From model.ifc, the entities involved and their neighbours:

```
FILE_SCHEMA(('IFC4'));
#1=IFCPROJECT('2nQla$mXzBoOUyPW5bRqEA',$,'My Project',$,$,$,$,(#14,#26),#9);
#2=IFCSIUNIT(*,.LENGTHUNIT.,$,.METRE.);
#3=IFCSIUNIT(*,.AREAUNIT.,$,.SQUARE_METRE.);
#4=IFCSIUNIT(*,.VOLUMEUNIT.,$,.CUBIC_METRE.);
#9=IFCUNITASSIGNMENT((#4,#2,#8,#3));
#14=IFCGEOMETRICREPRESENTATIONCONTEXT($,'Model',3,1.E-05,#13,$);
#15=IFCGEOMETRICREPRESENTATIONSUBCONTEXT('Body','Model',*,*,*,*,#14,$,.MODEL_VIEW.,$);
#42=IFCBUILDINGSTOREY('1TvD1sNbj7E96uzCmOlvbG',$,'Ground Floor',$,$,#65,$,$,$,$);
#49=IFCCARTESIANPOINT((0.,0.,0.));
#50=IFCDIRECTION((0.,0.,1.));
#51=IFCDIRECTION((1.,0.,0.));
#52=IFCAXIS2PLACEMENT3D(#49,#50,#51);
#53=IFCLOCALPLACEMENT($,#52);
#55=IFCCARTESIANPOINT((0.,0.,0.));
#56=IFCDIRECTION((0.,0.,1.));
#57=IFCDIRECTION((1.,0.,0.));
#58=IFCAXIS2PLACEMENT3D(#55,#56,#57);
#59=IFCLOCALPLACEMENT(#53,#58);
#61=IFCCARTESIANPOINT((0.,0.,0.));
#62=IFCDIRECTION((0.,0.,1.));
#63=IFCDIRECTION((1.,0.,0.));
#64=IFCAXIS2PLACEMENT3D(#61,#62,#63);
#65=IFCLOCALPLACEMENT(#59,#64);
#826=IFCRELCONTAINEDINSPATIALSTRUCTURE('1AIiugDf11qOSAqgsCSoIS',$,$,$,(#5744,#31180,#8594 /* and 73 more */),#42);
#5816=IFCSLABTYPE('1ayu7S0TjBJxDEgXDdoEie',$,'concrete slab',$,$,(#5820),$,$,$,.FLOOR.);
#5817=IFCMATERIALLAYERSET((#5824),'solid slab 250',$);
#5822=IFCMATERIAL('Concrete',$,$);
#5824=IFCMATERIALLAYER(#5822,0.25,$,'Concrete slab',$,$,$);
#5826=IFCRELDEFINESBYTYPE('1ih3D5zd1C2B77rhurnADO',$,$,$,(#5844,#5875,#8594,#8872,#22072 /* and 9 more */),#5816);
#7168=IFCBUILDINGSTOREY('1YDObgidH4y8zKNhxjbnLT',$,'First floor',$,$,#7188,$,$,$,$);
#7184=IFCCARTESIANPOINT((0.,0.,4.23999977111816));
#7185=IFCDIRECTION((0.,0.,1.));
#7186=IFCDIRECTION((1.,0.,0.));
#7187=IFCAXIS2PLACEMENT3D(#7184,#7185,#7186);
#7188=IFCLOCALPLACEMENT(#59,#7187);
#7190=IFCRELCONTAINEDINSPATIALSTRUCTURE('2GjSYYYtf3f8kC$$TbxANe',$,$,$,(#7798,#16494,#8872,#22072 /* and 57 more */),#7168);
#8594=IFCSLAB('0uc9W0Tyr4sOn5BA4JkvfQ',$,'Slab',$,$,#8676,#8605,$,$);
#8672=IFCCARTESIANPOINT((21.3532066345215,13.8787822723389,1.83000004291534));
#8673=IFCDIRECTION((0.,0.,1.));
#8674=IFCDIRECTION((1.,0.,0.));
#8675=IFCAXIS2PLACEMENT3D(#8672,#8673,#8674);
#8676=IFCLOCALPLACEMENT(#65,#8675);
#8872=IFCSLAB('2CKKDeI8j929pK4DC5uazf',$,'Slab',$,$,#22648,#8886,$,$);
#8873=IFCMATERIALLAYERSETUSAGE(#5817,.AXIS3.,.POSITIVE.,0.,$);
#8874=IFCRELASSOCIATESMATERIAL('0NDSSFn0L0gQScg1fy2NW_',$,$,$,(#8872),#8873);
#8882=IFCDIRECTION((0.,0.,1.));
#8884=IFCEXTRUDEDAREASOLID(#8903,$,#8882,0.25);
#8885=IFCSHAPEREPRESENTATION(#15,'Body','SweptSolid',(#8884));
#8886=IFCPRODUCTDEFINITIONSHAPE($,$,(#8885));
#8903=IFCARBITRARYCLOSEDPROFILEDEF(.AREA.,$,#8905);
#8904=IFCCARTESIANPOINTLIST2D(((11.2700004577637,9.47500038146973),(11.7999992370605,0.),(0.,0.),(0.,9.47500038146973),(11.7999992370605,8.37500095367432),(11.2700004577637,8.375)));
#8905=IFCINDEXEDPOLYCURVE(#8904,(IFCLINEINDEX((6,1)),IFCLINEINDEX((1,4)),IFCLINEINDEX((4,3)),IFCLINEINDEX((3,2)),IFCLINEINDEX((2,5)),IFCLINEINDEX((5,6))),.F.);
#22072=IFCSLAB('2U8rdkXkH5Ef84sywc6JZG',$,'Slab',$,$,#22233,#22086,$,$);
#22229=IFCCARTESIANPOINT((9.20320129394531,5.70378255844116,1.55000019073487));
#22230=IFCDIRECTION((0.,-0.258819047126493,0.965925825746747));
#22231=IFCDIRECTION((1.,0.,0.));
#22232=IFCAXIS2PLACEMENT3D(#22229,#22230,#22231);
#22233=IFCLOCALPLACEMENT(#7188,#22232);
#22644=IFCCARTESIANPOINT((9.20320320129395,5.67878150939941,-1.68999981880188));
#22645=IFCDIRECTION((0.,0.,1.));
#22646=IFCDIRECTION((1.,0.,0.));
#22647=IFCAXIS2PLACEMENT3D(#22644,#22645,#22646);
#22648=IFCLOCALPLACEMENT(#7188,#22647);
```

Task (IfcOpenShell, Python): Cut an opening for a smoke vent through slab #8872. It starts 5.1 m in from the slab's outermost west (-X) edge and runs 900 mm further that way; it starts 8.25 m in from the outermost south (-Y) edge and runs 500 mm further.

```python
import numpy as np
import ifcopenshell
import ifcopenshell.api.feature
import ifcopenshell.api.geometry
import ifcopenshell.api.root
import ifcopenshell.geom
import ifcopenshell.util.placement
import ifcopenshell.util.representation
import ifcopenshell.util.shape
import ifcopenshell.util.unit

model = ifcopenshell.open("model.ifc")
unit_scale = ifcopenshell.util.unit.calculate_unit_scale(model)
settings = ifcopenshell.geom.settings()


def volume(element):
    """Net volume in cubic metres, openings subtracted."""
    shape = ifcopenshell.geom.create_shape(settings, element)
    return ifcopenshell.util.shape.get_volume(shape.geometry)


slab = model.by_guid("2CKKDeI8j929pK4DC5uazf")
before = volume(slab)

# Extent in the slab's own axes, in metres. The edges named are its -X and -Y sides.
slab_shape = ifcopenshell.geom.create_shape(settings, slab)
vertices = ifcopenshell.util.shape.get_vertices(slab_shape.geometry)
x_min, y_min, bottom = vertices.min(axis=0)
top = vertices[:, 2].max()

opening = ifcopenshell.api.root.create_entity(model, ifc_class="IfcOpeningElement", name="Smoke vent opening", predefined_type="OPENING")
context = ifcopenshell.util.representation.get_context(model, "Model", "Body", "MODEL_VIEW")
width, depth = 0.9, 0.5
outline = [(0.0, 0.0), (width, 0.0), (width, depth), (0.0, depth), (0.0, 0.0)]
# Overshoot both faces by 50 mm so the cut is clean.
shape = ifcopenshell.api.geometry.add_slab_representation(
    model, context=context, depth=top - bottom + 0.1, polyline=outline
)
ifcopenshell.api.geometry.assign_representation(model, product=opening, representation=shape)

matrix = ifcopenshell.util.placement.get_local_placement(slab.ObjectPlacement)
matrix[:, 3] = matrix @ np.append(np.array([x_min + 5.1, y_min + 8.25, bottom - 0.05]) / unit_scale, 1.0)
ifcopenshell.api.geometry.edit_object_placement(model, product=opening, matrix=matrix, is_si=False)
ifcopenshell.api.feature.add_feature(model, feature=opening, element=slab)

after = volume(slab)

print(f"slab volume {before:.3f} -> {after:.3f} m3")

model.write("model-out.ifc")
```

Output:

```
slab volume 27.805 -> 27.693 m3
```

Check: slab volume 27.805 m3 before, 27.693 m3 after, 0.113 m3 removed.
